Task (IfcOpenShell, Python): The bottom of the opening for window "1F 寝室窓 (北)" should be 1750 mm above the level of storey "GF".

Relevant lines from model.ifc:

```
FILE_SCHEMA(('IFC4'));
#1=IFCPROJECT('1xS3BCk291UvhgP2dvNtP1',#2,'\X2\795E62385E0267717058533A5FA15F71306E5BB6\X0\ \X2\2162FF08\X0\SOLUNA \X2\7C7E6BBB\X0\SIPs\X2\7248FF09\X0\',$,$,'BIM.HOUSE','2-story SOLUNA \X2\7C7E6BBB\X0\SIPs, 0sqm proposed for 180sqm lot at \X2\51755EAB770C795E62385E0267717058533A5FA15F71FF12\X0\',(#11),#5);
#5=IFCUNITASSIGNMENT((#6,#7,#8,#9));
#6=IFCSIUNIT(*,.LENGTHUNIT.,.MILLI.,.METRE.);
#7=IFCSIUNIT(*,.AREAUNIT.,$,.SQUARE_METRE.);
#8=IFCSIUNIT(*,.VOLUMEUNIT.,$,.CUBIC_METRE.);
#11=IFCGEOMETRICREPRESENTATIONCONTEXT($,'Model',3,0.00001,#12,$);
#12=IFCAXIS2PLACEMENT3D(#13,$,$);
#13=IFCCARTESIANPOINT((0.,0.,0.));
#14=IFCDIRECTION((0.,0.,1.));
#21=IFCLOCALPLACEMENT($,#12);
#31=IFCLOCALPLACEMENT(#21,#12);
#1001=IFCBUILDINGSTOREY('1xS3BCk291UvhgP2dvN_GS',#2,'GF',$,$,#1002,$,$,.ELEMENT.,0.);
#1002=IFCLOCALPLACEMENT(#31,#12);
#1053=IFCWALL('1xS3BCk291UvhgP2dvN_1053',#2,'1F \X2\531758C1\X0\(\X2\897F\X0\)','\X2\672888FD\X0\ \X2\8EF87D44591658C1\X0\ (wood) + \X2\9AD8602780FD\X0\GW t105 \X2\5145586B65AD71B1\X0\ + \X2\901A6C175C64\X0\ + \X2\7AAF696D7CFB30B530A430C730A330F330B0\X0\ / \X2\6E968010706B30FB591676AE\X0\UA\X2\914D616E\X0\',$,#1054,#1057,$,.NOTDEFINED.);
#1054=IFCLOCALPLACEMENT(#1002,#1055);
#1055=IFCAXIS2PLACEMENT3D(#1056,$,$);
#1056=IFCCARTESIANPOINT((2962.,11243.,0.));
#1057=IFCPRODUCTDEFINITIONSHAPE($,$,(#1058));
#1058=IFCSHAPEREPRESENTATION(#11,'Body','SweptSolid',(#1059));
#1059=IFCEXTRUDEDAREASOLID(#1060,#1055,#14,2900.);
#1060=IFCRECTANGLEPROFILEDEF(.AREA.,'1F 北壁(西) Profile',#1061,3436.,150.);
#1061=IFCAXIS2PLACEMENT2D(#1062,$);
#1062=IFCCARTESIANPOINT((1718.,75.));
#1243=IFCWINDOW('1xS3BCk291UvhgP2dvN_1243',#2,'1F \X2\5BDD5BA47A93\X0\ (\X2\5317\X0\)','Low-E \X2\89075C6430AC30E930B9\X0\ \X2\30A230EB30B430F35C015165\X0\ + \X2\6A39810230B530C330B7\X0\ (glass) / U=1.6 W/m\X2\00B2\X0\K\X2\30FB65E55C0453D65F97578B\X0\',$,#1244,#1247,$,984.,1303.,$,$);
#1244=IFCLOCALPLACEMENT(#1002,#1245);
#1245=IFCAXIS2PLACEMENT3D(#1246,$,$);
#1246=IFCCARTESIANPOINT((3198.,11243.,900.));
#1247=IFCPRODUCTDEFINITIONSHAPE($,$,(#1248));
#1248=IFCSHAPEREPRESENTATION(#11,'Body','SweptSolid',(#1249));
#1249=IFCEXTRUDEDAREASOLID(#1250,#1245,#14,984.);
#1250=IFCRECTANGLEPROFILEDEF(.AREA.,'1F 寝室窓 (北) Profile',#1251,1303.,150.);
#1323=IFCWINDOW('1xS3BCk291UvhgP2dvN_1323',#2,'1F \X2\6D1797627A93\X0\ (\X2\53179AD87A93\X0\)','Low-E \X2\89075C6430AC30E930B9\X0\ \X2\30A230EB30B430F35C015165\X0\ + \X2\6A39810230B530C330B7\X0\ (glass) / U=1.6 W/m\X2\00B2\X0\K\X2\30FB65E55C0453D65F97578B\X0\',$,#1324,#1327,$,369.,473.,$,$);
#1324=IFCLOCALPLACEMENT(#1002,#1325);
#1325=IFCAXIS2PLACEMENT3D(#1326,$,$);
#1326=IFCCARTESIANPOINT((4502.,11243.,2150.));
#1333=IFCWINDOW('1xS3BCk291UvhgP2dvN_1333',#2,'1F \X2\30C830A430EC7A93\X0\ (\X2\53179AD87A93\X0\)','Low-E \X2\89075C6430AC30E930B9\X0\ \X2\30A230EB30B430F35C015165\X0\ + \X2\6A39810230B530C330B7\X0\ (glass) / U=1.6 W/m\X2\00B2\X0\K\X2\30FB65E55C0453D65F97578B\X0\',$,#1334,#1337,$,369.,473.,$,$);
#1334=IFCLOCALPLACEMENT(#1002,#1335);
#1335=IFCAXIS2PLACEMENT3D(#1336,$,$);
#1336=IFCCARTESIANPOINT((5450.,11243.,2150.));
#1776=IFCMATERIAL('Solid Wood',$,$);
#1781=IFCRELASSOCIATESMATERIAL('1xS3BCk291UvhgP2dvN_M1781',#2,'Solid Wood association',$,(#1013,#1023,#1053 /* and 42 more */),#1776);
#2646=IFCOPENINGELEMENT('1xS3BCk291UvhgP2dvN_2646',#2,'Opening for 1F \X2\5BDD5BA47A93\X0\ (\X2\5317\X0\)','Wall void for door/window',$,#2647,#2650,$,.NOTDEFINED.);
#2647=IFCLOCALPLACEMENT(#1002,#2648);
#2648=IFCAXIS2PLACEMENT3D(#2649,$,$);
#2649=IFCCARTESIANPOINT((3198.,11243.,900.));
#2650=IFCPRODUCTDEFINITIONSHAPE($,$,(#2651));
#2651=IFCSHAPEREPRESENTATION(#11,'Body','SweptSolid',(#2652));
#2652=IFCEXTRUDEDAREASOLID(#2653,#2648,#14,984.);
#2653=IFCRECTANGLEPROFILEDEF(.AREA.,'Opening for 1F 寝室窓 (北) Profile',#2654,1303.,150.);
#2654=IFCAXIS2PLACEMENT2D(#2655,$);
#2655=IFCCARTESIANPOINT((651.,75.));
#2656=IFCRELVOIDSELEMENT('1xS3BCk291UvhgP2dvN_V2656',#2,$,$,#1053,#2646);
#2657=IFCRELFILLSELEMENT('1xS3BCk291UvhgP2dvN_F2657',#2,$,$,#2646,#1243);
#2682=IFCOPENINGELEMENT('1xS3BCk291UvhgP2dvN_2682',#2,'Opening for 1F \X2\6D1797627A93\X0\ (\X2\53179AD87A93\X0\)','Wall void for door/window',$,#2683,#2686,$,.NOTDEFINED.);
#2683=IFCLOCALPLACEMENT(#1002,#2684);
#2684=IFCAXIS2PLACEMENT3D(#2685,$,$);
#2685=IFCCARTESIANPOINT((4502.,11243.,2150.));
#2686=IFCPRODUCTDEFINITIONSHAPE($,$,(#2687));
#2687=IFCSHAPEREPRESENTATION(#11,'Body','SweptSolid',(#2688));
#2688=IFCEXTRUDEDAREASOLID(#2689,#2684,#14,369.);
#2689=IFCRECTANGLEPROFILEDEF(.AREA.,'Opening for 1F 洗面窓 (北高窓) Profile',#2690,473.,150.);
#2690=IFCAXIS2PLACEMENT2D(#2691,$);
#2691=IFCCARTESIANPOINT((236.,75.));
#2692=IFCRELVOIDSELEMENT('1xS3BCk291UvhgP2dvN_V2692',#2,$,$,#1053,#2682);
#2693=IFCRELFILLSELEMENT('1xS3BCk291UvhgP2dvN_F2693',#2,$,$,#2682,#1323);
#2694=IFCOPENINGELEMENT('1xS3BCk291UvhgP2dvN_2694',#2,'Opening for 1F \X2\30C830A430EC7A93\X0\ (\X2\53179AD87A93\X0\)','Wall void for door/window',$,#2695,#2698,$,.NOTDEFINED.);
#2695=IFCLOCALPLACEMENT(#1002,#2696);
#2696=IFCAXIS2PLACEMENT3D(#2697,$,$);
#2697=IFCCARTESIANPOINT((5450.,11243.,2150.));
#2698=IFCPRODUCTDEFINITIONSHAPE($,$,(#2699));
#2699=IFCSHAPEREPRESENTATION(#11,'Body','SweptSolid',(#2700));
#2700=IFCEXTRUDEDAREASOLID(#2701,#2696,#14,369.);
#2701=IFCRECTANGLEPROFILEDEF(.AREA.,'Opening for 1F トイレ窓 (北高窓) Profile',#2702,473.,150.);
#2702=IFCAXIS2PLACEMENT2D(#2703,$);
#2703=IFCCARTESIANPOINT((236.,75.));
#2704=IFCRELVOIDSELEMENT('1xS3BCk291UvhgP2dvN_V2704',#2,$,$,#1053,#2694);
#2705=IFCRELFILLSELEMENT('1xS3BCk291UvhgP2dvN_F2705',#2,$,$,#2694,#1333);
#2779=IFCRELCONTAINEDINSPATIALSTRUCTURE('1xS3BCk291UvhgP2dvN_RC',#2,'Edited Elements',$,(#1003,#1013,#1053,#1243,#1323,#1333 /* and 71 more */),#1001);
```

```python
import numpy as np
import ifcopenshell
import ifcopenshell.api.geometry
import ifcopenshell.geom
import ifcopenshell.util.element
import ifcopenshell.util.placement
import ifcopenshell.util.shape
import ifcopenshell.util.unit

model = ifcopenshell.open("model.ifc")
unit_scale = ifcopenshell.util.unit.calculate_unit_scale(model)

window = model.by_guid("1xS3BCk291UvhgP2dvN_1243")
opening = window.FillsVoids[0].RelatingOpeningElement
storey = ifcopenshell.util.element.get_container(window, ifc_class="IfcBuildingStorey")
level = ifcopenshell.util.placement.get_local_placement(storey.ObjectPlacement)[2, 3]

# The opening's origin need not be at the sill, so measure its lowest point.
shape = ifcopenshell.geom.create_shape(ifcopenshell.geom.settings(), opening)
bottom = ifcopenshell.util.shape.get_shape_bottom_elevation(shape, shape.geometry) / unit_scale
dz = level + 1750.0 - bottom

shift = np.array([0.0, 0.0, dz])
# The window is not placed relative to its opening, so move both.
for product in (opening, window):
    matrix = ifcopenshell.util.placement.get_local_placement(product.ObjectPlacement)
    matrix[:3, 3] += shift
    ifcopenshell.api.geometry.edit_object_placement(model, product=product, matrix=matrix, is_si=False)

print(f"moved by {dz * unit_scale:+.3f} m")

model.write("model_edited.ifc")
```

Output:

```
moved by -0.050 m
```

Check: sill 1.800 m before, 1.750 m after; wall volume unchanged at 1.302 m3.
